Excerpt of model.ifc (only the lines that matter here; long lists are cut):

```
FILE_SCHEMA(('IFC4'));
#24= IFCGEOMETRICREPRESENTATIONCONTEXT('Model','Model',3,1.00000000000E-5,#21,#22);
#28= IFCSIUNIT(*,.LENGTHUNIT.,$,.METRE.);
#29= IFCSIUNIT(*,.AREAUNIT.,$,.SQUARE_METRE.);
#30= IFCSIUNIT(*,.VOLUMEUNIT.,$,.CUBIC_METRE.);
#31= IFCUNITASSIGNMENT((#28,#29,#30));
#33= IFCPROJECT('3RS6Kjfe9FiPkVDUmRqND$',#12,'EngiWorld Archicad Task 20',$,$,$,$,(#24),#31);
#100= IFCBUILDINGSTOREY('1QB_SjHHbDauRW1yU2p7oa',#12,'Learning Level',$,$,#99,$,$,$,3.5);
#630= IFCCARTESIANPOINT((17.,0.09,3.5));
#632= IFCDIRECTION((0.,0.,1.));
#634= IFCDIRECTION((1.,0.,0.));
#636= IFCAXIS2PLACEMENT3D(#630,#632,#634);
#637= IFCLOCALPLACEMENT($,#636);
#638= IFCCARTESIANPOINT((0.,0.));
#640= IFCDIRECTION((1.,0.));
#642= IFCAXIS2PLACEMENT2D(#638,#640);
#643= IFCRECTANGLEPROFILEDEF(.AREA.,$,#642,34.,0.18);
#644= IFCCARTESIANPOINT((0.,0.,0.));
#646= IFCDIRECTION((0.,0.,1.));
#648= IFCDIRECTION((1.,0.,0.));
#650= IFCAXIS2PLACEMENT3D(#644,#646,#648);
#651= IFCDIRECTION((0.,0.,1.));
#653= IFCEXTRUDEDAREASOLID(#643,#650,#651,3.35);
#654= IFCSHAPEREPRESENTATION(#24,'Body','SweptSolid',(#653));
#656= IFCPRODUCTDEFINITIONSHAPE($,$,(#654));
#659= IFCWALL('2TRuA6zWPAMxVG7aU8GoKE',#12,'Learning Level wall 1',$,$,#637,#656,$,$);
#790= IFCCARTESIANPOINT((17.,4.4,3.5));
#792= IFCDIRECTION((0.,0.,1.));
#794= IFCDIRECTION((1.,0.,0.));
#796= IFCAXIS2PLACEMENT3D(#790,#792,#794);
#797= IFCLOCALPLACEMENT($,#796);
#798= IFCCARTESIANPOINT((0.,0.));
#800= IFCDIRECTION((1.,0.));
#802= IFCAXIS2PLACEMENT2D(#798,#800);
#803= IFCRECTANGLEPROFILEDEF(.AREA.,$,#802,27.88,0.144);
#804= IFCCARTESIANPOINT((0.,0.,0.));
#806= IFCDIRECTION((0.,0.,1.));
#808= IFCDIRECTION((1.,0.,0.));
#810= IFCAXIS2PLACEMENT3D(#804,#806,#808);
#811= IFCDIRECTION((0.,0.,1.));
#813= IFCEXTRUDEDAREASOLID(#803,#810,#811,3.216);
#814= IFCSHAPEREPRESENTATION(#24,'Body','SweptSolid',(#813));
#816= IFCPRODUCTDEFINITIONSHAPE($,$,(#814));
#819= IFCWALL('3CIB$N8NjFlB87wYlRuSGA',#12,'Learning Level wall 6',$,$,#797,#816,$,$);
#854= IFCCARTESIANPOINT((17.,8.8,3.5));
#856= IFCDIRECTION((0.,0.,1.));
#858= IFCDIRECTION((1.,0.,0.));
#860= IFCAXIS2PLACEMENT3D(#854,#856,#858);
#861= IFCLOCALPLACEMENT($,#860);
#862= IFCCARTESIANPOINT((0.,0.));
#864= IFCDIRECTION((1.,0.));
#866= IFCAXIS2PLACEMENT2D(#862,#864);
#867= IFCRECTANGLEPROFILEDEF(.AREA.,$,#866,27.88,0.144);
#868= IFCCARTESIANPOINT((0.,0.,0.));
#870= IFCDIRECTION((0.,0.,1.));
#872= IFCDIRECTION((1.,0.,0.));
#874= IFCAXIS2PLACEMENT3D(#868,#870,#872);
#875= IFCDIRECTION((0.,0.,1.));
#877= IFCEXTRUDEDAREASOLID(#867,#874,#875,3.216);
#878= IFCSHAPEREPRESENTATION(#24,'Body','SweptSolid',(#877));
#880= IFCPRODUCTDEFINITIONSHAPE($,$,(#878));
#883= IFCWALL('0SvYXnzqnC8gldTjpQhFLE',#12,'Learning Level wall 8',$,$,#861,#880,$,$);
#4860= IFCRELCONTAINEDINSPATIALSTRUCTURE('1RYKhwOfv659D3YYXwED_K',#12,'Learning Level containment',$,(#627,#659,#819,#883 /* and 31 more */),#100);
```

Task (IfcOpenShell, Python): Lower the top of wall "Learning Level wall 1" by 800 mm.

```python
import ifcopenshell
import ifcopenshell.geom
import ifcopenshell.util.shape

model = ifcopenshell.open("model.ifc")
settings = ifcopenshell.geom.settings()


def volume(element):
    """Net volume in cubic metres, openings subtracted."""
    shape = ifcopenshell.geom.create_shape(settings, element)
    return ifcopenshell.util.shape.get_volume(shape.geometry)


wall = model.by_guid("2TRuA6zWPAMxVG7aU8GoKE")
before = volume(wall)

body = next(r for r in wall.Representation.Representations if r.RepresentationIdentifier == "Body")
solid = body.Items[0]
old_height = solid.Depth
solid.Depth -= 0.8
after = volume(wall)

print(f"height {old_height:g} -> {solid.Depth:g}, volume {before:.3f} -> {after:.3f} m3")

model.write("model_v2.ifc")
```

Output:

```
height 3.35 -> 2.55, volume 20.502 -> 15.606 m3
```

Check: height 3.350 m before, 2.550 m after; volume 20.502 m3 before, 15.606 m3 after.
